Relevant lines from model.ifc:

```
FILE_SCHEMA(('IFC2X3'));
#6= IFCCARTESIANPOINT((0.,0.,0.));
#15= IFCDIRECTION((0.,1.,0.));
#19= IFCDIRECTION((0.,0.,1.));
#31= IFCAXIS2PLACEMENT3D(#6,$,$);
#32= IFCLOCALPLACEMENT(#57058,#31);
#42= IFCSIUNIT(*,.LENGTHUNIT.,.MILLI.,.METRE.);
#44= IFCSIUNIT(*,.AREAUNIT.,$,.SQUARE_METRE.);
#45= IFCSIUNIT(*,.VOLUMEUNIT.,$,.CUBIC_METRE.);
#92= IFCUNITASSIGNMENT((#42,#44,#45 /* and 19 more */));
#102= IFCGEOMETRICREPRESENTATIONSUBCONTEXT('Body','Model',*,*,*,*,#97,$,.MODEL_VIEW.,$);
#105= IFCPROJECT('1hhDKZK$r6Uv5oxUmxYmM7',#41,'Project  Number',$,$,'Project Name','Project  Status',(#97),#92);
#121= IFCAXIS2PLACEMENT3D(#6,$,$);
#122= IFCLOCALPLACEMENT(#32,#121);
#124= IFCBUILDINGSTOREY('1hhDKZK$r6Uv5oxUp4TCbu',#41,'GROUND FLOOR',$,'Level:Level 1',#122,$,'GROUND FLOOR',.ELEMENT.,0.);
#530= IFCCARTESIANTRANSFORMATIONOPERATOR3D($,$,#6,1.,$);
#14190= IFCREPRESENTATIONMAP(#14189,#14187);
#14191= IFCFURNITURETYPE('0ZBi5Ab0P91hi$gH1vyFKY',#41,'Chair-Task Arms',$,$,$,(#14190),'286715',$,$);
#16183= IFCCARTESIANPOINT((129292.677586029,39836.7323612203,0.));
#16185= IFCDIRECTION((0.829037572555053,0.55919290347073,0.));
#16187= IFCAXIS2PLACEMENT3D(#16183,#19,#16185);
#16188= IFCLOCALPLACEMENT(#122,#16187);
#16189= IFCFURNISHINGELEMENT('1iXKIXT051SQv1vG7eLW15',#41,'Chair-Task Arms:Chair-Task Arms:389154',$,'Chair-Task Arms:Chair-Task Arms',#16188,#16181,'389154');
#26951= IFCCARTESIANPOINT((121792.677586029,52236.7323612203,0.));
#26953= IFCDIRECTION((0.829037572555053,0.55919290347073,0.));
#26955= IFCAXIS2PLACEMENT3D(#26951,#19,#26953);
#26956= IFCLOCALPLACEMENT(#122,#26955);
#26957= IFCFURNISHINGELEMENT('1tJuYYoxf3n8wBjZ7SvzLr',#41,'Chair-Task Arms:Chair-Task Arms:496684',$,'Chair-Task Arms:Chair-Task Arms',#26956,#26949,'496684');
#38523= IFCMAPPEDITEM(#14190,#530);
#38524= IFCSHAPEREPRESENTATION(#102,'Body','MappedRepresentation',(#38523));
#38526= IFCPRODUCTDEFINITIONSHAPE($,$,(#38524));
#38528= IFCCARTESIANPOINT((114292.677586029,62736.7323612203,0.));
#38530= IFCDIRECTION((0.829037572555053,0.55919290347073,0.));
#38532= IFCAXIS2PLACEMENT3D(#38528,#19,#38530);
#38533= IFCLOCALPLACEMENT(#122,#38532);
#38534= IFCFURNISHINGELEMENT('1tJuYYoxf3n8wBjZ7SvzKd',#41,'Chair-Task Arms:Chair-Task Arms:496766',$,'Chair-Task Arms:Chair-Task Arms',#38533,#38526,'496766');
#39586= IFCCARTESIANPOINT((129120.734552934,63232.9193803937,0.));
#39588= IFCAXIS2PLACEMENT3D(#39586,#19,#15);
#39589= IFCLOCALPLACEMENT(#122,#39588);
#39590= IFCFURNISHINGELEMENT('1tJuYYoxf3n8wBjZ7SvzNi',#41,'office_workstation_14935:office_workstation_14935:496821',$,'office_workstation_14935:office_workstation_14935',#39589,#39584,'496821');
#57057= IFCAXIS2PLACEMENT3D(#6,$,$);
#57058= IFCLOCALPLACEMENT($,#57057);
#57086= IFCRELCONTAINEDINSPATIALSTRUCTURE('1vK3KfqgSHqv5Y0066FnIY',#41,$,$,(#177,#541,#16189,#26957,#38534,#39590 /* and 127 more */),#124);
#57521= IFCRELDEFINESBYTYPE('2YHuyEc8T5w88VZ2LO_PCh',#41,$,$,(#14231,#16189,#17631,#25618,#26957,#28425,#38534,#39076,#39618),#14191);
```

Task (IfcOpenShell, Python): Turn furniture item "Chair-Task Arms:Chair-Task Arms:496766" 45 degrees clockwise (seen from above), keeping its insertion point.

```python
import ifcopenshell
import ifcopenshell.api.geometry
import ifcopenshell.util.placement

model = ifcopenshell.open("model.ifc")

item = model.by_id(38534)
matrix = ifcopenshell.util.placement.get_local_placement(item.ObjectPlacement)
matrix = matrix @ ifcopenshell.util.placement.rotation(-45, "Z")
ifcopenshell.api.geometry.edit_object_placement(model, product=item, matrix=matrix, is_si=False)

print(ifcopenshell.util.placement.get_local_placement(item.ObjectPlacement).round(3) + 0.0)

model.write("model_edited.ifc")
```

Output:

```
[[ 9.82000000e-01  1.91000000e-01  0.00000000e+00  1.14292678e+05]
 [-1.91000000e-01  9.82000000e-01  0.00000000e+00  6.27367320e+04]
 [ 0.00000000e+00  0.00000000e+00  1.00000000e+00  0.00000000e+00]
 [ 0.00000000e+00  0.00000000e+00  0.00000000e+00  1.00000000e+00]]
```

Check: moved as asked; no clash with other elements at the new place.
